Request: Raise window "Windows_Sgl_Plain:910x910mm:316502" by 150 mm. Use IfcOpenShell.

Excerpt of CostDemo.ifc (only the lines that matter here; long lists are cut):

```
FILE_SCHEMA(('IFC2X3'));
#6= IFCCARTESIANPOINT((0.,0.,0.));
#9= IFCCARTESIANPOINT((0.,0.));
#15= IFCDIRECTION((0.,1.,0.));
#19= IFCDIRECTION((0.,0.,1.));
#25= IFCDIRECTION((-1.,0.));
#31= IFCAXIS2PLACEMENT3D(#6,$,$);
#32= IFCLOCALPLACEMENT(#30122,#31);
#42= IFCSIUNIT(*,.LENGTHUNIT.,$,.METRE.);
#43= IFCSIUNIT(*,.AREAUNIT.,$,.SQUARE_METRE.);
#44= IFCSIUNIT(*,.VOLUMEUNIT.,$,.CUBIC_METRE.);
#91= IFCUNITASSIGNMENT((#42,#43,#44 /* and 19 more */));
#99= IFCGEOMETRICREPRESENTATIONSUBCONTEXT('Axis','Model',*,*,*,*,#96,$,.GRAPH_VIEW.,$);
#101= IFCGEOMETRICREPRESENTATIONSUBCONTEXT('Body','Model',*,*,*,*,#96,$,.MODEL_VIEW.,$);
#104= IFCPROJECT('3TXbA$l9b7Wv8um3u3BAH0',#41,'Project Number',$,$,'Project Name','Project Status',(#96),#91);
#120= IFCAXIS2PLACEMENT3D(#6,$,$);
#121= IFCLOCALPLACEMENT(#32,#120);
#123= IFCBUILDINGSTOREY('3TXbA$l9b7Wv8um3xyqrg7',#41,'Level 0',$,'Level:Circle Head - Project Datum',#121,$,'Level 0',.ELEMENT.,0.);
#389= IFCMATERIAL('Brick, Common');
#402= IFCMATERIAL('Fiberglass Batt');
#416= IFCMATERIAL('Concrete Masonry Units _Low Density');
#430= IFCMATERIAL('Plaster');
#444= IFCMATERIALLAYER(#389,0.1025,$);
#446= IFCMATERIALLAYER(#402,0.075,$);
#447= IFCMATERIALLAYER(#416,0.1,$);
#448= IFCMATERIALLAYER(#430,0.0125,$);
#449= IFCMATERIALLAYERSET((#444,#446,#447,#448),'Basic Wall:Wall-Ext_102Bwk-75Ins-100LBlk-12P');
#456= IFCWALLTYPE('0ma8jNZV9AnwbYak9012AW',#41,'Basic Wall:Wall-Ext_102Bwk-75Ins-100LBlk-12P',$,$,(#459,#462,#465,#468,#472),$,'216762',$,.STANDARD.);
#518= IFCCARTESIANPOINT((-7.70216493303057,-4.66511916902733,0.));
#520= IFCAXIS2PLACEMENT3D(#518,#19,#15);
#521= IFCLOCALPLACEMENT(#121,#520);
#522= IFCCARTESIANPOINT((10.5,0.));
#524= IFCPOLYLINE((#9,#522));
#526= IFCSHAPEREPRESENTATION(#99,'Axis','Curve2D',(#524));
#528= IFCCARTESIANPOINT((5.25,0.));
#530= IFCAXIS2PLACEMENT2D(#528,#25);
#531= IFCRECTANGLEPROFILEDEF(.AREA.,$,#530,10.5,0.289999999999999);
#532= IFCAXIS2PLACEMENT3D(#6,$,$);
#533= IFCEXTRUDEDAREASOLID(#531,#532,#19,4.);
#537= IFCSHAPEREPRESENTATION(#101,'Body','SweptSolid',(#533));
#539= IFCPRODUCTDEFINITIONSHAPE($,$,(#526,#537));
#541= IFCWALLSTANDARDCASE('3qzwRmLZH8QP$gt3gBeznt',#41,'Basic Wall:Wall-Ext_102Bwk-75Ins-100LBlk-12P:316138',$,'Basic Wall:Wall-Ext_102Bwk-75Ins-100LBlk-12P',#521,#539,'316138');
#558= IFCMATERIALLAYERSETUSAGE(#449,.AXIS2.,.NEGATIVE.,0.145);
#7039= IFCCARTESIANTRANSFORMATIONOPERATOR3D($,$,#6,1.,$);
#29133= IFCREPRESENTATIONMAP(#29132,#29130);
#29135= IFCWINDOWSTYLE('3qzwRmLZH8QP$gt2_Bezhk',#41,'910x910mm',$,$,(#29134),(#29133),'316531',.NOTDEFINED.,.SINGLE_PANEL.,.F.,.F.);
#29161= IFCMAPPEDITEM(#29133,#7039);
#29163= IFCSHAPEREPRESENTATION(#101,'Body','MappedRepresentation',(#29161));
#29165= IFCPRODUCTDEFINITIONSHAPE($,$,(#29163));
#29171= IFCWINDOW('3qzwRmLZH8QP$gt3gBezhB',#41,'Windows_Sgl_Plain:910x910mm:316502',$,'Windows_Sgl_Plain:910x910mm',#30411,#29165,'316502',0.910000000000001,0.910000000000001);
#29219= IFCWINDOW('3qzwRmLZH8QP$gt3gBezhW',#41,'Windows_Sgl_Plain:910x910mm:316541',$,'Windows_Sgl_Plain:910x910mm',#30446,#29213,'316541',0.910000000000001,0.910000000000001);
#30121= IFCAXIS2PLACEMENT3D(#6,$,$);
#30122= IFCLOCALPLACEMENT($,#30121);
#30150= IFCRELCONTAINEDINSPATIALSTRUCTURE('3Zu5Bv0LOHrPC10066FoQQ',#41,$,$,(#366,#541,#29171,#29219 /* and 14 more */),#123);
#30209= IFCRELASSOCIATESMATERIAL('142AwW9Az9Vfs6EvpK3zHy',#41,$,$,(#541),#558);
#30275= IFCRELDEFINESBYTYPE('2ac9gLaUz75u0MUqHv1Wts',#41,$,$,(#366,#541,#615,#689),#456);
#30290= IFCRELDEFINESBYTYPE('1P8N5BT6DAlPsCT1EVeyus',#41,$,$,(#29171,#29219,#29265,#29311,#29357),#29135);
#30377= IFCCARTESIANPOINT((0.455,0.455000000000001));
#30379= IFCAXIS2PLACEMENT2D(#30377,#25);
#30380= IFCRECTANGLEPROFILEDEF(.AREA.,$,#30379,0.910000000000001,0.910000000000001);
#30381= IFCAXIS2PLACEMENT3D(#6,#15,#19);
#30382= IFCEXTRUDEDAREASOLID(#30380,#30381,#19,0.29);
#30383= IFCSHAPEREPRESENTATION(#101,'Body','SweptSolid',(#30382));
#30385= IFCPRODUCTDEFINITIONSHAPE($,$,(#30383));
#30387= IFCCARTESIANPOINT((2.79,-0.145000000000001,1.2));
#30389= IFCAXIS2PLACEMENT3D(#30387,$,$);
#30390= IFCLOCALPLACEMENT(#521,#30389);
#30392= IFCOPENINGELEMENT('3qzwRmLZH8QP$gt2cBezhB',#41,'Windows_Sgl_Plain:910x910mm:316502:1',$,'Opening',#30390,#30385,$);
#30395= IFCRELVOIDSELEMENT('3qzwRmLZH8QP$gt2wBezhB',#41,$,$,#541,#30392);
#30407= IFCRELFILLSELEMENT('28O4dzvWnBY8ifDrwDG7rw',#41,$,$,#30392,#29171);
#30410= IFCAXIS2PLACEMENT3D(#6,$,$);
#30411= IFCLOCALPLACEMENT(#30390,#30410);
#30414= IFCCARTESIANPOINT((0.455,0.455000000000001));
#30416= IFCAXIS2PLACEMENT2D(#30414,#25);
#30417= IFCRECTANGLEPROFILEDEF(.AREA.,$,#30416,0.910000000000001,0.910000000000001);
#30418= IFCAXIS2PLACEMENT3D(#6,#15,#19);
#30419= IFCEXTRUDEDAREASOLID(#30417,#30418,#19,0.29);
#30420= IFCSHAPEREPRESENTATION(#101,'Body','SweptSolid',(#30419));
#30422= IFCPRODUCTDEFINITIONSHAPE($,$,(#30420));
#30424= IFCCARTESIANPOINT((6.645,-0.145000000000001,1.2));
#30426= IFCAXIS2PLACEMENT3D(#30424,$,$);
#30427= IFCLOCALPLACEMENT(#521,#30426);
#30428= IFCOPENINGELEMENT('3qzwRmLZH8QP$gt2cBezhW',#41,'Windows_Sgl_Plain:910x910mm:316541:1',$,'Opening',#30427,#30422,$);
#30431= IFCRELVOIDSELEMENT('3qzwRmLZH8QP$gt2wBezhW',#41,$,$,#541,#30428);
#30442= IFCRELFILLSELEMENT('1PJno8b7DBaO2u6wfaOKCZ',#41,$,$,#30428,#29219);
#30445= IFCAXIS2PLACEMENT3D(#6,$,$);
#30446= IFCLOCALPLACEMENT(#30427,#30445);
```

```python
import numpy as np
import ifcopenshell
import ifcopenshell.api.geometry
import ifcopenshell.util.placement
import ifcopenshell.util.unit

model = ifcopenshell.open("CostDemo.ifc")
unit_scale = ifcopenshell.util.unit.calculate_unit_scale(model)

window = model.by_guid("3qzwRmLZH8QP$gt3gBezhB")
opening = window.FillsVoids[0].RelatingOpeningElement
dz = 0.15

shift = np.array([0.0, 0.0, dz])
# The window is placed relative to its opening, so it follows when the opening moves.
matrix = ifcopenshell.util.placement.get_local_placement(opening.ObjectPlacement)
matrix[:3, 3] += shift
ifcopenshell.api.geometry.edit_object_placement(
    model, product=opening, matrix=matrix, is_si=False, should_transform_children=True
)

print(f"moved by {dz * unit_scale:+.3f} m")

model.write("CostDemo_v2.ifc")
```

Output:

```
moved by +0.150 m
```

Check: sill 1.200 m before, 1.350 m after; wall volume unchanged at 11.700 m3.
